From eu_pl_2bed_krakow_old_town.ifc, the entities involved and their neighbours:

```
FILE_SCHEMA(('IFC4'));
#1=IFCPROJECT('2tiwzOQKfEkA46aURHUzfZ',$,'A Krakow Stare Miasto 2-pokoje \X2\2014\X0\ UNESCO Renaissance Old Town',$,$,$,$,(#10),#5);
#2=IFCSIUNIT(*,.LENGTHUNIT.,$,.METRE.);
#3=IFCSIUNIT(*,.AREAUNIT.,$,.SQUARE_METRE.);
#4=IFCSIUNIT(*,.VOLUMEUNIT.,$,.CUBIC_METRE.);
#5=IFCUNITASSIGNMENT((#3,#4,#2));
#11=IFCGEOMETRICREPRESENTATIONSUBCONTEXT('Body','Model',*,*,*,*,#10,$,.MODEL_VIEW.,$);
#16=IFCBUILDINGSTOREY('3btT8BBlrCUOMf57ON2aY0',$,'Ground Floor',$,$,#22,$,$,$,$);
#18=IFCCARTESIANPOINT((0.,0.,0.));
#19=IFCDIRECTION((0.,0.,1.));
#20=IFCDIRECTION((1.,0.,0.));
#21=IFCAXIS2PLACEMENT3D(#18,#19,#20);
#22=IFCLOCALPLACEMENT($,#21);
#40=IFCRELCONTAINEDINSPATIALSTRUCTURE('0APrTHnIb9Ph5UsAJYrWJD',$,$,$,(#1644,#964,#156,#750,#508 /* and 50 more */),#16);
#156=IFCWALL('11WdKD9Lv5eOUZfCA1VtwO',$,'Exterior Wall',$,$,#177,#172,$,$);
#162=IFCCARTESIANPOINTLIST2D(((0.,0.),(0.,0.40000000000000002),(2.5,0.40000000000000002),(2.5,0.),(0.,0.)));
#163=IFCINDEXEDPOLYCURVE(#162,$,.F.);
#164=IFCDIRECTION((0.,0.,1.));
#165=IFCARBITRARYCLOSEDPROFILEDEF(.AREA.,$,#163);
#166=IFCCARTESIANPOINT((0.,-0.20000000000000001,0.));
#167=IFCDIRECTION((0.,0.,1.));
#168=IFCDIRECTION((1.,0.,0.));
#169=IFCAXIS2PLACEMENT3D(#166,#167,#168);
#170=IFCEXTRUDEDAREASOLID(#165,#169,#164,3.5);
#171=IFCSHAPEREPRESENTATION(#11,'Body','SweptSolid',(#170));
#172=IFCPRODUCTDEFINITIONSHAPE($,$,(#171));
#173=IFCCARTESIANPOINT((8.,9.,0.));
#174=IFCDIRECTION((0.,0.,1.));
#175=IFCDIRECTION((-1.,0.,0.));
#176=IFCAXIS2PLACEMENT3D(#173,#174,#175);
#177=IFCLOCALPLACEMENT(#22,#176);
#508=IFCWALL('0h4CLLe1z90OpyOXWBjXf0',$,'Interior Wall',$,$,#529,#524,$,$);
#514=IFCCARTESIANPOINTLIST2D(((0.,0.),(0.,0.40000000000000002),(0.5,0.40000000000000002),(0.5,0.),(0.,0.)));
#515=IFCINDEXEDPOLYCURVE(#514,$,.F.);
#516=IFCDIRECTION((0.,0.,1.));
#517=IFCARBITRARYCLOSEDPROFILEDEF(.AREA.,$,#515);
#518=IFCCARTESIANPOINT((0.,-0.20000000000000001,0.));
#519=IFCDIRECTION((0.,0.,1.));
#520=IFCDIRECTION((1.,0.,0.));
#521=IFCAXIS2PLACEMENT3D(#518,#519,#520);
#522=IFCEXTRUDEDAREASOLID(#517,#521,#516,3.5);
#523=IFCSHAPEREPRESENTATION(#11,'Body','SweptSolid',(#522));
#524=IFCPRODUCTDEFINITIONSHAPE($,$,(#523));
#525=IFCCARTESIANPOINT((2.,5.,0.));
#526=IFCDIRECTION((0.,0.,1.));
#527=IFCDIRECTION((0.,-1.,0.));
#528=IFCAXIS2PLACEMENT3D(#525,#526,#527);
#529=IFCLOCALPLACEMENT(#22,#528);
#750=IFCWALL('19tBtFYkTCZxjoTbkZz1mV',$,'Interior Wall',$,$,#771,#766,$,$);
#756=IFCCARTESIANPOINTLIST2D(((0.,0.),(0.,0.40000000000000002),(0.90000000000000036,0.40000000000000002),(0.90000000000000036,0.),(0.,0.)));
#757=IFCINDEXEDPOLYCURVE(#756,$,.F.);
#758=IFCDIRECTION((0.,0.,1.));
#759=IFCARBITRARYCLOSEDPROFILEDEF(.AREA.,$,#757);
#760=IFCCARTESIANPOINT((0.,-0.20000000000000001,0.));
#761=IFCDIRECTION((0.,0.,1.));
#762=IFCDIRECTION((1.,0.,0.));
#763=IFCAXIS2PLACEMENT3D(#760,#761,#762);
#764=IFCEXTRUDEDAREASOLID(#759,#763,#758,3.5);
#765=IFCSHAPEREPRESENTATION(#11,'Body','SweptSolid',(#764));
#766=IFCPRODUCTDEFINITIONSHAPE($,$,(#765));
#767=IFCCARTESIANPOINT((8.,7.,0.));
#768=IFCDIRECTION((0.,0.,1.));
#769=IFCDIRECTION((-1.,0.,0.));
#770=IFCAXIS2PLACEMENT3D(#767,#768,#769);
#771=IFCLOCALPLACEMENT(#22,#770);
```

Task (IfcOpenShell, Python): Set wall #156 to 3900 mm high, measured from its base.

```python
import ifcopenshell
import ifcopenshell.geom
import ifcopenshell.util.representation
import ifcopenshell.util.shape

model = ifcopenshell.open("eu_pl_2bed_krakow_old_town.ifc")
settings = ifcopenshell.geom.settings()


def volume(element):
    """Net volume in cubic metres, openings subtracted."""
    shape = ifcopenshell.geom.create_shape(settings, element)
    return ifcopenshell.util.shape.get_volume(shape.geometry)


wall = model.by_guid("11WdKD9Lv5eOUZfCA1VtwO")
before = volume(wall)

body = ifcopenshell.util.representation.get_representation(wall, "Model", "Body")
solid = body.Items[0]
old_height = solid.Depth
solid.Depth = 3.9
after = volume(wall)

print(f"height {old_height:g} -> {solid.Depth:g}, volume {before:.3f} -> {after:.3f} m3")

model.write("eu_pl_2bed_krakow_old_town_rev.ifc")
```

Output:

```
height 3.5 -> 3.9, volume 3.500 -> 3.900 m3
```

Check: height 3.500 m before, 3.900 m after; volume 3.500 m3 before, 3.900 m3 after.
